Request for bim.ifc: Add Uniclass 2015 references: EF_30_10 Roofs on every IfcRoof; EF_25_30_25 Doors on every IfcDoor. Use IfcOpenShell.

First a look at what the model holds.

```python
import ifcopenshell

model = ifcopenshell.open("bim.ifc")
print(model.schema)
print("classifications:", [c.Name for c in model.by_type("IfcClassification")])
for ifc_class in ("IfcDoor", "IfcRoof", "IfcStair", "IfcWall", "IfcWindow"):
    print(ifc_class, len(model.by_type(ifc_class)))
```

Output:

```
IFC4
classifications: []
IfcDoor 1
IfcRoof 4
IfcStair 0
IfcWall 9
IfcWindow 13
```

```python
import ifcopenshell
import ifcopenshell.api.classification

model = ifcopenshell.open("bim.ifc")

system = ifcopenshell.api.classification.add_classification(model, classification="Uniclass 2015")

codes = {
    "IfcRoof": ("EF_30_10", "Roofs"),
    "IfcDoor": ("EF_25_30_25", "Doors"),
}
for ifc_class, (code, name) in codes.items():
    products = model.by_type(ifc_class)
    ifcopenshell.api.classification.add_reference(
        model, products=products, classification=system, identification=code, name=name
    )
    print(code, len(products))

model.write("bim_v2.ifc")
```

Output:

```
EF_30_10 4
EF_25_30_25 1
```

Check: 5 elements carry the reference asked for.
